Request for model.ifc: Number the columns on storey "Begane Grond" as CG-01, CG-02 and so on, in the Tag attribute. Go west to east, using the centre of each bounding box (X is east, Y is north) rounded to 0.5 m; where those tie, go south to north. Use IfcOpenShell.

First a look at what the model holds.

```python
import ifcopenshell
import ifcopenshell.util.element
import ifcopenshell.util.placement

model = ifcopenshell.open("model.ifc")
print(model.schema)
storey = next(s for s in model.by_type("IfcBuildingStorey") if s.Name == "Begane Grond")
columns = [e for e in ifcopenshell.util.element.get_decomposition(storey) if e.is_a("IfcColumn")]
for e in sorted(columns, key=lambda e: e.id()):
    origin = ifcopenshell.util.placement.get_local_placement(e.ObjectPlacement)[:3, 3]
    print(e.id(), e.Tag, e.Name, origin.round(2) + 0.0, sep=" | ")
```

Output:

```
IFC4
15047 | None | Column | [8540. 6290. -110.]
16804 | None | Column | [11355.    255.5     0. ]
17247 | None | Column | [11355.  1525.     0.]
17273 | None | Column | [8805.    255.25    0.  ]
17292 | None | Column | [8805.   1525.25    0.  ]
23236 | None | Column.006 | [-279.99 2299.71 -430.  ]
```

```python
import ifcopenshell
import ifcopenshell.geom
import ifcopenshell.util.element
import ifcopenshell.util.shape

model = ifcopenshell.open("model.ifc")
settings = ifcopenshell.geom.settings()
settings.set("use-world-coords", True)


def centre(element):
    shape = ifcopenshell.geom.create_shape(settings, element)
    return ifcopenshell.util.shape.get_bbox_centroid(shape.geometry)


storey = next(s for s in model.by_type("IfcBuildingStorey") if s.Name == "Begane Grond")
columns = [e for e in ifcopenshell.util.element.get_decomposition(storey) if e.is_a("IfcColumn")]

# Insertion points can sit at a corner or the storey origin, so sort by the geometry (in metres).
centres = {e: centre(e) for e in columns}
columns.sort(key=lambda e: (round(centres[e][0] / 0.5), centres[e][1]))

for i, e in enumerate(columns, start=1):
    number = f"CG-{i:02d}"
    e.Tag = number
    print(e.id(), number)

model.write("model_edited.ifc")
```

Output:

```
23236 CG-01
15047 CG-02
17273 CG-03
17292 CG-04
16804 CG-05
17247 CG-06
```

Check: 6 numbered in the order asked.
